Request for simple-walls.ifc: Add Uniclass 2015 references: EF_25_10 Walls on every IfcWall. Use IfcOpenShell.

First a look at what the model holds.

```python
import ifcopenshell

model = ifcopenshell.open("simple-walls.ifc")
print(model.schema)
print("classifications:", [c.Name for c in model.by_type("IfcClassification")])
for ifc_class in ("IfcDoor", "IfcRoof", "IfcStair", "IfcWall", "IfcWindow"):
    print(ifc_class, len(model.by_type(ifc_class)))
```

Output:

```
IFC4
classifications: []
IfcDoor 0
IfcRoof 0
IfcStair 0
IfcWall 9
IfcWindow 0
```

```python
import ifcopenshell
import ifcopenshell.api.classification

model = ifcopenshell.open("simple-walls.ifc")

system = ifcopenshell.api.classification.add_classification(model, classification="Uniclass 2015")

codes = {
    "IfcWall": ("EF_25_10", "Walls"),
}
for ifc_class, (code, name) in codes.items():
    products = model.by_type(ifc_class)
    ifcopenshell.api.classification.add_reference(
        model, products=products, classification=system, identification=code, name=name
    )
    print(code, len(products))

model.write("simple-walls_v2.ifc")
```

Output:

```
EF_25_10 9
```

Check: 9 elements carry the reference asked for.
